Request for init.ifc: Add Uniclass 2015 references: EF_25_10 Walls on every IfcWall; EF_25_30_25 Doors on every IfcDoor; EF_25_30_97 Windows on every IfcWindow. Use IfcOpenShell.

First a look at what the model holds.

```python
import ifcopenshell

model = ifcopenshell.open("init.ifc")
print(model.schema)
print("classifications:", [c.Name for c in model.by_type("IfcClassification")])
for ifc_class in ("IfcDoor", "IfcRoof", "IfcStair", "IfcWall", "IfcWindow"):
    print(ifc_class, len(model.by_type(ifc_class)))
```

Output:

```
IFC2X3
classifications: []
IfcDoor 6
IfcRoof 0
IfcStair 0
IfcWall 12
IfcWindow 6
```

```python
import ifcopenshell
import ifcopenshell.api.classification

model = ifcopenshell.open("init.ifc")

# IFC2X3 requires Source and Edition and has no link from the project to the system.
system = model.create_entity("IfcClassification", Source="NBS", Edition="2015", Name="Uniclass 2015")

codes = {
    "IfcWall": ("EF_25_10", "Walls"),
    "IfcDoor": ("EF_25_30_25", "Doors"),
    "IfcWindow": ("EF_25_30_97", "Windows"),
}
for ifc_class, (code, name) in codes.items():
    products = model.by_type(ifc_class)
    ifcopenshell.api.classification.add_reference(
        model, products=products, classification=system, identification=code, name=name
    )
    print(code, len(products))

model.write("init_v2.ifc")
```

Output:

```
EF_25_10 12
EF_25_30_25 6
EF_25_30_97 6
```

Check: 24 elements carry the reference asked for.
